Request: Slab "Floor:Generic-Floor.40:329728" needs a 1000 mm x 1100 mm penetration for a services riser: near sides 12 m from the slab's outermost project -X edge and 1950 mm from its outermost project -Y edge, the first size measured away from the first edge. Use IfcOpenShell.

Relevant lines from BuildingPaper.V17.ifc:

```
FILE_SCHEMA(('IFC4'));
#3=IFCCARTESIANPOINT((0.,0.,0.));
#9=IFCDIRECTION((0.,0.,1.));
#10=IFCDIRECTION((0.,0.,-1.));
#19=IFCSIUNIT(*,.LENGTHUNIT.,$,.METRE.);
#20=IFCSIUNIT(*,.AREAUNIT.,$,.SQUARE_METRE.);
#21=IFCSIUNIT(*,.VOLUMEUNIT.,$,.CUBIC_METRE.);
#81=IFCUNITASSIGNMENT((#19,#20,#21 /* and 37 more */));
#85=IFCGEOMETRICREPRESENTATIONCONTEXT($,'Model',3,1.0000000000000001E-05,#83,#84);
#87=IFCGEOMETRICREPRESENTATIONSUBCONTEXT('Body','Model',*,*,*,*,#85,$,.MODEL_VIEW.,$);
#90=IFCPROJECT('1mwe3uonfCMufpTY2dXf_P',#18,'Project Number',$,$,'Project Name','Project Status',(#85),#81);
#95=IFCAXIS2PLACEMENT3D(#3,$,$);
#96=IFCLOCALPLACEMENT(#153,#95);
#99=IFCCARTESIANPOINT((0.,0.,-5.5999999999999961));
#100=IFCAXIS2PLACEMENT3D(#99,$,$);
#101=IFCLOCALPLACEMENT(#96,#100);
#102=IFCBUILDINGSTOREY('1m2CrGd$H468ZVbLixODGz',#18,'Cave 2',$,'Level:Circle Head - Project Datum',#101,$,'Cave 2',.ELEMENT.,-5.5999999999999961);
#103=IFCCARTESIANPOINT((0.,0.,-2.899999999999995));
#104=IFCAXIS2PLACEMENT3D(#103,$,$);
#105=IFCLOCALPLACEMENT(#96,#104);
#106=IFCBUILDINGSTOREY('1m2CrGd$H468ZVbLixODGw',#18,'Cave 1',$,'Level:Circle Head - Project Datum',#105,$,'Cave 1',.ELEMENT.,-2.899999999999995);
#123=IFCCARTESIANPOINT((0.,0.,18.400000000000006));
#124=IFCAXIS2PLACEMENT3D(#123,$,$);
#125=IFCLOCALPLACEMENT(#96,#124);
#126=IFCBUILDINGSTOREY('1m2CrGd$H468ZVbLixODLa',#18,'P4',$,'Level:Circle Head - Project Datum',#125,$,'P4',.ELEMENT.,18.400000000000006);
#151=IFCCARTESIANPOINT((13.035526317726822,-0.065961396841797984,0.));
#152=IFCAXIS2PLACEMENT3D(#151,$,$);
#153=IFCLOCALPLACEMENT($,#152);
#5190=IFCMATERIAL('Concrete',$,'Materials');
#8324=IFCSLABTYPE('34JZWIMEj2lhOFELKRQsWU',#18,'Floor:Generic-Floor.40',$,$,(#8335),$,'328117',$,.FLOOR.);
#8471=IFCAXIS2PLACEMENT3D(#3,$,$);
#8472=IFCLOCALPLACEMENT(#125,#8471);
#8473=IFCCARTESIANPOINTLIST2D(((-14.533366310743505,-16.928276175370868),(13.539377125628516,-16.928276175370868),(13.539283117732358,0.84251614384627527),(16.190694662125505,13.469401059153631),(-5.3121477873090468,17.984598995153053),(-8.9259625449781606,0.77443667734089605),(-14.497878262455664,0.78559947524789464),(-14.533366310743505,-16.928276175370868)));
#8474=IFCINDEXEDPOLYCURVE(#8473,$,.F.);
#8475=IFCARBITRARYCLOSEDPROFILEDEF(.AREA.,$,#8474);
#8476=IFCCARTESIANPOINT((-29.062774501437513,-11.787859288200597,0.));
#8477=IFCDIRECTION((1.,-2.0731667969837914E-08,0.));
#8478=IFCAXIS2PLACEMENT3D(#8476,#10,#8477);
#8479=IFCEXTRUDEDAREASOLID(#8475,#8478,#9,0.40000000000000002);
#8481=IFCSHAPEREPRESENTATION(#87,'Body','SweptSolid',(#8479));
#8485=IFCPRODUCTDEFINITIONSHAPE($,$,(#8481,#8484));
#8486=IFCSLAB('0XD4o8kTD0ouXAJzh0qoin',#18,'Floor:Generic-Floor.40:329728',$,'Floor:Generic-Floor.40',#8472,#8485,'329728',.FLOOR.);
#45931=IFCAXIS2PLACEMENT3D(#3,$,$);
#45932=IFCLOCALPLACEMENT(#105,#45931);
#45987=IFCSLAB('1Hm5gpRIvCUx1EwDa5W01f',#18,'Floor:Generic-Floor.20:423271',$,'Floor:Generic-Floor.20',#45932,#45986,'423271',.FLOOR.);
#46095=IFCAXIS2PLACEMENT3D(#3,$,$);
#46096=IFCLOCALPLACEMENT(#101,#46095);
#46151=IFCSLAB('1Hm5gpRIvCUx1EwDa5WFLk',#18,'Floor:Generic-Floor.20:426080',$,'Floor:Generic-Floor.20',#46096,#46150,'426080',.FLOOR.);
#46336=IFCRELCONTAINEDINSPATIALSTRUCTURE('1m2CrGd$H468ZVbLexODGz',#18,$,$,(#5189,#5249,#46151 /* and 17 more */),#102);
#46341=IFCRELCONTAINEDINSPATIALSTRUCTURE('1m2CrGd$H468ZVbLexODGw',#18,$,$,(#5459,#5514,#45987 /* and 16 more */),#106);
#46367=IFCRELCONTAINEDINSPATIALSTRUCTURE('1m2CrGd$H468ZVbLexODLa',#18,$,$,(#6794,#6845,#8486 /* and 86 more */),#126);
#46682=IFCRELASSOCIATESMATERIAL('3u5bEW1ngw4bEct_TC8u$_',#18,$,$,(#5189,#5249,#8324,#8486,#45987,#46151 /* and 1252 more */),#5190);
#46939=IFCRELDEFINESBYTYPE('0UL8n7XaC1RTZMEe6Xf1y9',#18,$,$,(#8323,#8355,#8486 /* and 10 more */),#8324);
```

```python
import numpy as np
import ifcopenshell
import ifcopenshell.api.feature
import ifcopenshell.api.geometry
import ifcopenshell.api.root
import ifcopenshell.geom
import ifcopenshell.util.placement
import ifcopenshell.util.representation
import ifcopenshell.util.shape
import ifcopenshell.util.unit

model = ifcopenshell.open("BuildingPaper.V17.ifc")
unit_scale = ifcopenshell.util.unit.calculate_unit_scale(model)
settings = ifcopenshell.geom.settings()


def volume(element):
    """Net volume in cubic metres, openings subtracted."""
    shape = ifcopenshell.geom.create_shape(settings, element)
    return ifcopenshell.util.shape.get_volume(shape.geometry)


slab = model.by_guid("0XD4o8kTD0ouXAJzh0qoin")
before = volume(slab)

# Extent in the slab's own axes, in metres. The edges named are its -X and -Y sides.
slab_shape = ifcopenshell.geom.create_shape(settings, slab)
vertices = ifcopenshell.util.shape.get_vertices(slab_shape.geometry)
x_min, y_min, bottom = vertices.min(axis=0)
top = vertices[:, 2].max()

opening = ifcopenshell.api.root.create_entity(model, ifc_class="IfcOpeningElement", name="Services riser opening", predefined_type="OPENING")
context = ifcopenshell.util.representation.get_context(model, "Model", "Body", "MODEL_VIEW")
width, depth = 1, 1.1
outline = [(0.0, 0.0), (width, 0.0), (width, depth), (0.0, depth), (0.0, 0.0)]
# Overshoot both faces by 50 mm so the cut is clean.
shape = ifcopenshell.api.geometry.add_slab_representation(
    model, context=context, depth=top - bottom + 0.1, polyline=outline
)
ifcopenshell.api.geometry.assign_representation(model, product=opening, representation=shape)

matrix = ifcopenshell.util.placement.get_local_placement(slab.ObjectPlacement)
matrix[:, 3] = matrix @ np.append(np.array([x_min + 12, y_min + 1.95, bottom - 0.05]) / unit_scale, 1.0)
ifcopenshell.api.geometry.edit_object_placement(model, product=opening, matrix=matrix, is_si=False)
ifcopenshell.api.feature.add_feature(model, feature=opening, element=slab)

after = volume(slab)

print(f"slab volume {before:.3f} -> {after:.3f} m3")

model.write("BuildingPaper.V17-out.ifc")
```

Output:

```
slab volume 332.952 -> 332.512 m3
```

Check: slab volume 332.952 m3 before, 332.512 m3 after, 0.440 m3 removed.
